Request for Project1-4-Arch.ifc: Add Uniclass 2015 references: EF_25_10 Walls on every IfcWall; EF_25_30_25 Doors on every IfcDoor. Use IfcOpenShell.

First a look at what the model holds.

```python
import ifcopenshell

model = ifcopenshell.open("Project1-4-Arch.ifc")
print(model.schema)
print("classifications:", [c.Name for c in model.by_type("IfcClassification")])
for ifc_class in ("IfcDoor", "IfcRoof", "IfcStair", "IfcWall", "IfcWindow"):
    print(ifc_class, len(model.by_type(ifc_class)))
```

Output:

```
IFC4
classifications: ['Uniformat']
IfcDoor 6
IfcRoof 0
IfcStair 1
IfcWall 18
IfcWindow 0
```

```python
import ifcopenshell
import ifcopenshell.api.classification

model = ifcopenshell.open("Project1-4-Arch.ifc")

system = ifcopenshell.api.classification.add_classification(model, classification="Uniclass 2015")

codes = {
    "IfcWall": ("EF_25_10", "Walls"),
    "IfcDoor": ("EF_25_30_25", "Doors"),
}
for ifc_class, (code, name) in codes.items():
    products = model.by_type(ifc_class)
    ifcopenshell.api.classification.add_reference(
        model, products=products, classification=system, identification=code, name=name
    )
    print(code, len(products))

model.write("Project1-4-Arch_v2.ifc")
```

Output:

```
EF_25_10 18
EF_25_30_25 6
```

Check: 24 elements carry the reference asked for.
